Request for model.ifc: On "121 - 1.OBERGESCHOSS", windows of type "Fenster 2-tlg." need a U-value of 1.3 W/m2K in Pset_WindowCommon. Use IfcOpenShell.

First a look at what the model holds.

```python
import ifcopenshell
import ifcopenshell.util.element

model = ifcopenshell.open("model.ifc")
print(model.schema)
storey = next(s for s in model.by_type("IfcBuildingStorey") if s.Name == "121 - 1.OBERGESCHOSS")
windows = [e for e in ifcopenshell.util.element.get_decomposition(storey) if e.is_a("IfcWindow")]
seen = {}
for e in windows:
    element_type = ifcopenshell.util.element.get_type(e)
    key = (element_type.Name if element_type != e and element_type else None, ifcopenshell.util.element.get_pset(e, "Pset_WindowCommon", "ThermalTransmittance"))
    seen[key] = seen.get(key, 0) + 1
for (name, value), count in sorted(seen.items(), key=str):
    print(count, "x", name, "|", value)
```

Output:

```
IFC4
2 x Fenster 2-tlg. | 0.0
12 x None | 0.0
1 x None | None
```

```python
import ifcopenshell
import ifcopenshell.api.pset
import ifcopenshell.util.element

model = ifcopenshell.open("model.ifc")

storey = next(s for s in model.by_type("IfcBuildingStorey") if s.Name == "121 - 1.OBERGESCHOSS")
windows = [e for e in ifcopenshell.util.element.get_decomposition(storey) if e.is_a("IfcWindow")]

count = 0
for e in windows:
    element_type = ifcopenshell.util.element.get_type(e)
    if element_type in (None, e) or element_type.Name != "Fenster 2-tlg.":
        continue
    # add_pset returns the element's existing set when there is one.
    pset = ifcopenshell.api.pset.add_pset(model, product=e, name="Pset_WindowCommon")
    ifcopenshell.api.pset.edit_pset(model, pset=pset, properties={"ThermalTransmittance": 1.3})
    count += 1

print(count, "windows updated")

model.write("model_updated.ifc")
```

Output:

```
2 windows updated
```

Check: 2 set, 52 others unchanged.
